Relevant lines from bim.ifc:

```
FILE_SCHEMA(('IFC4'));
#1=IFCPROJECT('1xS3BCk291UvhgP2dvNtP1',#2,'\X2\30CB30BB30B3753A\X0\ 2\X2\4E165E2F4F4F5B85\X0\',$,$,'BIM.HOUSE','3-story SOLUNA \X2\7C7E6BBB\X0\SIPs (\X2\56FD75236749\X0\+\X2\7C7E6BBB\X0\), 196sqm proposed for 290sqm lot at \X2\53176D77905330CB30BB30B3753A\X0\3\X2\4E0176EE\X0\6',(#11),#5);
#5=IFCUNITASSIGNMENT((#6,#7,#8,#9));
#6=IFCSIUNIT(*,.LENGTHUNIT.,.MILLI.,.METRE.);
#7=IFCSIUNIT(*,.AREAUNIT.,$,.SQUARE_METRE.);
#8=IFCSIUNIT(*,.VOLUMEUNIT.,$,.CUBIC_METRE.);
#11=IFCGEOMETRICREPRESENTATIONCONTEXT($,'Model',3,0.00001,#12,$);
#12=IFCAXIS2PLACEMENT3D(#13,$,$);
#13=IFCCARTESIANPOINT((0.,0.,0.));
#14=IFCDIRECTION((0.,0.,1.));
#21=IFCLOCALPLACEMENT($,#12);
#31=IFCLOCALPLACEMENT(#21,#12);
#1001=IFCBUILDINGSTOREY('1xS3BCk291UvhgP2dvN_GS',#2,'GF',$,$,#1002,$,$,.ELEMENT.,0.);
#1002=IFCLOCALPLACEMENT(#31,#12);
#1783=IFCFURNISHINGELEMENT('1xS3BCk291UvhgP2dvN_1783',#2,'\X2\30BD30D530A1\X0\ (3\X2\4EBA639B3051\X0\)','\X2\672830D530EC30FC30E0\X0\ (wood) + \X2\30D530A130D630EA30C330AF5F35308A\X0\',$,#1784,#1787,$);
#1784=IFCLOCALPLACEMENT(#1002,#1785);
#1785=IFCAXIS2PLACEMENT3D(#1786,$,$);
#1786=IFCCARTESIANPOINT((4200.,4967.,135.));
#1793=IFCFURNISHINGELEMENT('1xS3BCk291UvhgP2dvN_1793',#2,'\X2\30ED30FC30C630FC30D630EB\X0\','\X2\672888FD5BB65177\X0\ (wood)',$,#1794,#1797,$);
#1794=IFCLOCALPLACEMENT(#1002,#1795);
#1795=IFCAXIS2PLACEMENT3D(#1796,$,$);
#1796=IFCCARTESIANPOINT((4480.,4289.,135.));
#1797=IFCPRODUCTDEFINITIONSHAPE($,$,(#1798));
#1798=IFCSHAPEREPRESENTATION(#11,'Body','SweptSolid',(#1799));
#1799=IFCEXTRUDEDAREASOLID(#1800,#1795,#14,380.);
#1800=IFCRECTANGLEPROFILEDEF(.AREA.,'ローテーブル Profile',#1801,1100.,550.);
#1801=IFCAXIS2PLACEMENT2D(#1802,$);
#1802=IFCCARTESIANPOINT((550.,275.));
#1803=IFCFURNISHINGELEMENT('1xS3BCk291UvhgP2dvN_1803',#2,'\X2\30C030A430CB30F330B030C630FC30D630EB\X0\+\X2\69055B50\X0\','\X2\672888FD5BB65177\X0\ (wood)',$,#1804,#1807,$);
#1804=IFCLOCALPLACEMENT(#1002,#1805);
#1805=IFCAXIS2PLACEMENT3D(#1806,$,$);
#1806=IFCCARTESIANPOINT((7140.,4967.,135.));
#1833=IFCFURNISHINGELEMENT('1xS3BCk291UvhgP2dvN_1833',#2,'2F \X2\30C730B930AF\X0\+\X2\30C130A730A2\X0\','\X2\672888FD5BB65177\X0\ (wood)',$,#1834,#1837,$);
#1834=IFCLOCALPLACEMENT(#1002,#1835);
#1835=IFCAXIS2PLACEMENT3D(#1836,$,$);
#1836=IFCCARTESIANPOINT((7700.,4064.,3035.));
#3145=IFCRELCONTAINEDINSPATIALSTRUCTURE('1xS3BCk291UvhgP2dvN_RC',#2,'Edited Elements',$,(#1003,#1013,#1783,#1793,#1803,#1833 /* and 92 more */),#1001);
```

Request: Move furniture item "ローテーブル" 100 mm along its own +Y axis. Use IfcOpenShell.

```python
import ifcopenshell
import ifcopenshell.api.geometry
import ifcopenshell.util.placement
import ifcopenshell.util.unit

model = ifcopenshell.open("bim.ifc")
unit_scale = ifcopenshell.util.unit.calculate_unit_scale(model)

item = model.by_guid("1xS3BCk291UvhgP2dvN_1793")
matrix = ifcopenshell.util.placement.get_local_placement(item.ObjectPlacement)
matrix[:3, 3] += matrix[:3, 1] * 0.1 / unit_scale
ifcopenshell.api.geometry.edit_object_placement(model, product=item, matrix=matrix, is_si=False)

print(ifcopenshell.util.placement.get_local_placement(item.ObjectPlacement).round(3) + 0.0)

model.write("bim-out.ifc")
```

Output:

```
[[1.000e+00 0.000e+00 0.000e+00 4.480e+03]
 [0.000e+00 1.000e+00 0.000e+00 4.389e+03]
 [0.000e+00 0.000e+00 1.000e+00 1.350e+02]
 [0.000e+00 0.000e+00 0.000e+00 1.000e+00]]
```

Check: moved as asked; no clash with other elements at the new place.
